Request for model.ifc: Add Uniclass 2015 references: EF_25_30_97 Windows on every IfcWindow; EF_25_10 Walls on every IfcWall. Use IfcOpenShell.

First a look at what the model holds.

```python
import ifcopenshell

model = ifcopenshell.open("model.ifc")
print(model.schema)
print("classifications:", [c.Name for c in model.by_type("IfcClassification")])
for ifc_class in ("IfcDoor", "IfcRoof", "IfcStair", "IfcWall", "IfcWindow"):
    print(ifc_class, len(model.by_type(ifc_class)))
```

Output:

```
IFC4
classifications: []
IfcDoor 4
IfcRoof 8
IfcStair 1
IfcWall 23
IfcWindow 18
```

```python
import ifcopenshell
import ifcopenshell.api.classification

model = ifcopenshell.open("model.ifc")

system = ifcopenshell.api.classification.add_classification(model, classification="Uniclass 2015")

codes = {
    "IfcWindow": ("EF_25_30_97", "Windows"),
    "IfcWall": ("EF_25_10", "Walls"),
}
for ifc_class, (code, name) in codes.items():
    products = model.by_type(ifc_class)
    ifcopenshell.api.classification.add_reference(
        model, products=products, classification=system, identification=code, name=name
    )
    print(code, len(products))

model.write("model-out.ifc")
```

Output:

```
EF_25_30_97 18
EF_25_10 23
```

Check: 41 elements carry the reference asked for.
